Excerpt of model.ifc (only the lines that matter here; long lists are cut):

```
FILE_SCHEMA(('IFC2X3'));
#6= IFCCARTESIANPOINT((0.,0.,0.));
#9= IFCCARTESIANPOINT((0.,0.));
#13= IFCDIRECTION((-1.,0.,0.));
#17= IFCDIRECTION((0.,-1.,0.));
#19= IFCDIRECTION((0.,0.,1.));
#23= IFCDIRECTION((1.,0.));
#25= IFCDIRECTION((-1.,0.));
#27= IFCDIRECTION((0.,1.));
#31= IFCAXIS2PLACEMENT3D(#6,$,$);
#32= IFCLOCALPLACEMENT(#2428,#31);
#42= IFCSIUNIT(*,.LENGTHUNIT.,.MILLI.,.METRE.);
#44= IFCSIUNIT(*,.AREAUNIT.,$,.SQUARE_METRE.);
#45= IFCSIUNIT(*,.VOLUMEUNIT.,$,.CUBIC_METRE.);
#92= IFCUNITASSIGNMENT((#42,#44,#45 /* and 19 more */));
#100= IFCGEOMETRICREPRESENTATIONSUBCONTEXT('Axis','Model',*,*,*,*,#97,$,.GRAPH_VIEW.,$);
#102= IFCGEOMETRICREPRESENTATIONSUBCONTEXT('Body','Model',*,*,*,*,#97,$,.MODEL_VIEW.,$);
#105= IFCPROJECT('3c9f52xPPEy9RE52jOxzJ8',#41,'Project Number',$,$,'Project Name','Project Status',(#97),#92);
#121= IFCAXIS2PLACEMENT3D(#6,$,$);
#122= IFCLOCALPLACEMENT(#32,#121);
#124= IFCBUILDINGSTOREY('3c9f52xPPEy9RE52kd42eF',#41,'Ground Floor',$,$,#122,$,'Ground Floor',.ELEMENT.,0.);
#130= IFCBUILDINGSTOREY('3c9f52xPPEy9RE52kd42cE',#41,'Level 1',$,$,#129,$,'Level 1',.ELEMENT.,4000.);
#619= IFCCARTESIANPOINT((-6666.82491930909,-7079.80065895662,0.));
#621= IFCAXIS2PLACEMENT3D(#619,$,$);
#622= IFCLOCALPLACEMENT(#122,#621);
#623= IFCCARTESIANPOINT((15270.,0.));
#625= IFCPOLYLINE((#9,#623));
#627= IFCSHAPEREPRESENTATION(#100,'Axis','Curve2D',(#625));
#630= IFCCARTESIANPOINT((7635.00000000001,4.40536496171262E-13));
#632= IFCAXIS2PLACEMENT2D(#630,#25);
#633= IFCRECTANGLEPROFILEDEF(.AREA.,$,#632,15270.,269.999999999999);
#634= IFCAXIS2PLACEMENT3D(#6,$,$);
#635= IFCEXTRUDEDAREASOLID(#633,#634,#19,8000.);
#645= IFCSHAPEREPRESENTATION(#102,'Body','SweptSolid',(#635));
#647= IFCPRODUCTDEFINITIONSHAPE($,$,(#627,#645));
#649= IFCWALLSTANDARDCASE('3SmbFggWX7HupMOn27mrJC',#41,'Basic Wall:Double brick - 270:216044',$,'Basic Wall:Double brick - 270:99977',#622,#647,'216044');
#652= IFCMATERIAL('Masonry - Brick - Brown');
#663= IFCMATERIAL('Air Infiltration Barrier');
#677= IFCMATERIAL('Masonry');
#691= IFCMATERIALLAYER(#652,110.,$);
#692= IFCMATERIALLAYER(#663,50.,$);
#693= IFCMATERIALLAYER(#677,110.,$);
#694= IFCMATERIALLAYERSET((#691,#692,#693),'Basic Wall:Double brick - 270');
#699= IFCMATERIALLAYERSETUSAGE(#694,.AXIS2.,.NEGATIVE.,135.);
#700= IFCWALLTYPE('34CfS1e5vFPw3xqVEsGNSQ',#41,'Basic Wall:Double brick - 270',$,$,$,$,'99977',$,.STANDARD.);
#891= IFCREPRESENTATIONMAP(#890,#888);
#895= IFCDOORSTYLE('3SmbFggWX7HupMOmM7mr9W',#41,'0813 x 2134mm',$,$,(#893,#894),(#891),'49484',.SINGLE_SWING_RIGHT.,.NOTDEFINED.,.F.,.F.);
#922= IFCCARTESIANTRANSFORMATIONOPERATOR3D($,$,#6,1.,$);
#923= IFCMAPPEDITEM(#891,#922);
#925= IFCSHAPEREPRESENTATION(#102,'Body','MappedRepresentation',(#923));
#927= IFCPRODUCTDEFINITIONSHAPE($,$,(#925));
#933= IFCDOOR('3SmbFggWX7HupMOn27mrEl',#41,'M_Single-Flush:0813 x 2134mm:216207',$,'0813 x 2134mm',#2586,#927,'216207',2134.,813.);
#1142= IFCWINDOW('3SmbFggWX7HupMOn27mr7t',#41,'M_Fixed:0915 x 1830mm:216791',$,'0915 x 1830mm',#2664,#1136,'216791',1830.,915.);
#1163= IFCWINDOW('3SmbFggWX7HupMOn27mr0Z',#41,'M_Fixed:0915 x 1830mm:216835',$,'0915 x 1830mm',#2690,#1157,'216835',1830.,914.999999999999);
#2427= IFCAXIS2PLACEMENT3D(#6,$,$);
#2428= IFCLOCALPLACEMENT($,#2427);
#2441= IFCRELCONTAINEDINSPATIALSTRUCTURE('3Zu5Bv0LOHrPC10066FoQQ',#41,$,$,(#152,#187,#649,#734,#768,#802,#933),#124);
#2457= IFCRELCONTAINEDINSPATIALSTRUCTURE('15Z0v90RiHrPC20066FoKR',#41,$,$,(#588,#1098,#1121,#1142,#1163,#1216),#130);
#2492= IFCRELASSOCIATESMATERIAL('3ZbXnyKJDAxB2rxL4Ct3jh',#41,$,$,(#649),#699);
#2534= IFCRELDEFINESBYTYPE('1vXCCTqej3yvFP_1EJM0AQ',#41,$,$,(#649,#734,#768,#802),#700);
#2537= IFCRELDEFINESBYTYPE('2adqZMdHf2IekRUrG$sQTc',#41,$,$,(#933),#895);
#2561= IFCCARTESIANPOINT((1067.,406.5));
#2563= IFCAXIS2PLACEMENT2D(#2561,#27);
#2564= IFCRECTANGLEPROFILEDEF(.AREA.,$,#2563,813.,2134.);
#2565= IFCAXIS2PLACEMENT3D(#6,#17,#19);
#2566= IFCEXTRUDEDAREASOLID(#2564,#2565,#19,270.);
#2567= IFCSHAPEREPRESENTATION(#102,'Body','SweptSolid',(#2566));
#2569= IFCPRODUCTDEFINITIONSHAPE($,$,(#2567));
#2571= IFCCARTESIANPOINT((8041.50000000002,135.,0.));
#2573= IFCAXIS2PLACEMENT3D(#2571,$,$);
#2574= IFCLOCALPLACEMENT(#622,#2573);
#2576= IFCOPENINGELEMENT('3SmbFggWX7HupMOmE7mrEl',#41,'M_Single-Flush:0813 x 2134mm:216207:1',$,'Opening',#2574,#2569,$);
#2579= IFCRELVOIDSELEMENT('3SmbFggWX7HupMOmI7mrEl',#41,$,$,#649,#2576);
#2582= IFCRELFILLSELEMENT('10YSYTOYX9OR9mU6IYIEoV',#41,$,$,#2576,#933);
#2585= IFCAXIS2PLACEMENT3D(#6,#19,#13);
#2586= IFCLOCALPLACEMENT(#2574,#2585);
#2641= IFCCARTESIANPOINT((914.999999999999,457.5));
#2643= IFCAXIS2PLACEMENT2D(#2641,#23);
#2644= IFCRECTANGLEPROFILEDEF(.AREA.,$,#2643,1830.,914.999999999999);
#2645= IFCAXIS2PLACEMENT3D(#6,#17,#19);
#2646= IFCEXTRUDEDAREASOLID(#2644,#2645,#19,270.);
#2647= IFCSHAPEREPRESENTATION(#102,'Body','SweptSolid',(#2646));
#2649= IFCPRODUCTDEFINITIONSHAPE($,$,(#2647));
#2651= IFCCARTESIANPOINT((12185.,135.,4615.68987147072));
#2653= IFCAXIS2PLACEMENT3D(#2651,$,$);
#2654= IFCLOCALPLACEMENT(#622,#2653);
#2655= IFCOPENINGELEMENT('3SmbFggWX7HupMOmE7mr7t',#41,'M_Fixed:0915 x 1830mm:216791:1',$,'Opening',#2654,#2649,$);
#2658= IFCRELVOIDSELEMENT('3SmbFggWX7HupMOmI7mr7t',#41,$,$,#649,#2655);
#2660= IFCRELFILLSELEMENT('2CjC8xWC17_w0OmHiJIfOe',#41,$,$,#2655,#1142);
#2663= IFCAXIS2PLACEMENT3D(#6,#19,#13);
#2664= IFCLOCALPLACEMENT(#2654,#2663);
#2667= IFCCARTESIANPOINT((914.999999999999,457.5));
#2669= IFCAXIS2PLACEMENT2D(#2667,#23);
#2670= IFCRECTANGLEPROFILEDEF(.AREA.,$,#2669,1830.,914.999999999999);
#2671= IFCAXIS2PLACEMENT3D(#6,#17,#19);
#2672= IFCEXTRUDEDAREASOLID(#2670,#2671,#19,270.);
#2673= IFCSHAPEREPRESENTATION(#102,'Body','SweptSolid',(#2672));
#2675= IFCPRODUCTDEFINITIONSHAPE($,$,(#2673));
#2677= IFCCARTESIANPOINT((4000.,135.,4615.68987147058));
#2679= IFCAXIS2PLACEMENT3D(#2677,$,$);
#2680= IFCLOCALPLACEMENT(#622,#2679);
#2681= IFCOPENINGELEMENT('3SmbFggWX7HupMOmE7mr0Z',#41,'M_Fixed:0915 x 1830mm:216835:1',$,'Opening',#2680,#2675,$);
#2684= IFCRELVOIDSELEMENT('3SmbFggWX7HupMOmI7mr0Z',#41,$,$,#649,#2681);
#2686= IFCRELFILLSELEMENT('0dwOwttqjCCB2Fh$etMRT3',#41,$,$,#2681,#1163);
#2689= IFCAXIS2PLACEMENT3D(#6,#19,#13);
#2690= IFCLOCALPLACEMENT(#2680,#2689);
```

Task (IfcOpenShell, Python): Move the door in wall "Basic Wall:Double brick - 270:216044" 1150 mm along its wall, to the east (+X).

```python
import ifcopenshell
import ifcopenshell.api.geometry
import ifcopenshell.util.placement

model = ifcopenshell.open("model.ifc")

door = model.by_id(933)
opening = door.FillsVoids[0].RelatingOpeningElement
wall = opening.VoidsElements[0].RelatingBuildingElement

wall_matrix = ifcopenshell.util.placement.get_local_placement(wall.ObjectPlacement)
shift = wall_matrix[:3, 0] * 1150.0
before = ifcopenshell.util.placement.get_local_placement(door.ObjectPlacement)[:3, 3].copy()

# The door is placed relative to its opening, so it follows when the opening moves.
matrix = ifcopenshell.util.placement.get_local_placement(opening.ObjectPlacement)
matrix[:3, 3] += shift
ifcopenshell.api.geometry.edit_object_placement(
    model, product=opening, matrix=matrix, is_si=False, should_transform_children=True
)

after = ifcopenshell.util.placement.get_local_placement(door.ObjectPlacement)[:3, 3]
print("door moved by", (after - before).round(3) + 0.0)

model.write("model_edited.ifc")
```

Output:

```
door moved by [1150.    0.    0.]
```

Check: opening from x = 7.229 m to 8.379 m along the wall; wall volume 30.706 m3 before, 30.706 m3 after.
